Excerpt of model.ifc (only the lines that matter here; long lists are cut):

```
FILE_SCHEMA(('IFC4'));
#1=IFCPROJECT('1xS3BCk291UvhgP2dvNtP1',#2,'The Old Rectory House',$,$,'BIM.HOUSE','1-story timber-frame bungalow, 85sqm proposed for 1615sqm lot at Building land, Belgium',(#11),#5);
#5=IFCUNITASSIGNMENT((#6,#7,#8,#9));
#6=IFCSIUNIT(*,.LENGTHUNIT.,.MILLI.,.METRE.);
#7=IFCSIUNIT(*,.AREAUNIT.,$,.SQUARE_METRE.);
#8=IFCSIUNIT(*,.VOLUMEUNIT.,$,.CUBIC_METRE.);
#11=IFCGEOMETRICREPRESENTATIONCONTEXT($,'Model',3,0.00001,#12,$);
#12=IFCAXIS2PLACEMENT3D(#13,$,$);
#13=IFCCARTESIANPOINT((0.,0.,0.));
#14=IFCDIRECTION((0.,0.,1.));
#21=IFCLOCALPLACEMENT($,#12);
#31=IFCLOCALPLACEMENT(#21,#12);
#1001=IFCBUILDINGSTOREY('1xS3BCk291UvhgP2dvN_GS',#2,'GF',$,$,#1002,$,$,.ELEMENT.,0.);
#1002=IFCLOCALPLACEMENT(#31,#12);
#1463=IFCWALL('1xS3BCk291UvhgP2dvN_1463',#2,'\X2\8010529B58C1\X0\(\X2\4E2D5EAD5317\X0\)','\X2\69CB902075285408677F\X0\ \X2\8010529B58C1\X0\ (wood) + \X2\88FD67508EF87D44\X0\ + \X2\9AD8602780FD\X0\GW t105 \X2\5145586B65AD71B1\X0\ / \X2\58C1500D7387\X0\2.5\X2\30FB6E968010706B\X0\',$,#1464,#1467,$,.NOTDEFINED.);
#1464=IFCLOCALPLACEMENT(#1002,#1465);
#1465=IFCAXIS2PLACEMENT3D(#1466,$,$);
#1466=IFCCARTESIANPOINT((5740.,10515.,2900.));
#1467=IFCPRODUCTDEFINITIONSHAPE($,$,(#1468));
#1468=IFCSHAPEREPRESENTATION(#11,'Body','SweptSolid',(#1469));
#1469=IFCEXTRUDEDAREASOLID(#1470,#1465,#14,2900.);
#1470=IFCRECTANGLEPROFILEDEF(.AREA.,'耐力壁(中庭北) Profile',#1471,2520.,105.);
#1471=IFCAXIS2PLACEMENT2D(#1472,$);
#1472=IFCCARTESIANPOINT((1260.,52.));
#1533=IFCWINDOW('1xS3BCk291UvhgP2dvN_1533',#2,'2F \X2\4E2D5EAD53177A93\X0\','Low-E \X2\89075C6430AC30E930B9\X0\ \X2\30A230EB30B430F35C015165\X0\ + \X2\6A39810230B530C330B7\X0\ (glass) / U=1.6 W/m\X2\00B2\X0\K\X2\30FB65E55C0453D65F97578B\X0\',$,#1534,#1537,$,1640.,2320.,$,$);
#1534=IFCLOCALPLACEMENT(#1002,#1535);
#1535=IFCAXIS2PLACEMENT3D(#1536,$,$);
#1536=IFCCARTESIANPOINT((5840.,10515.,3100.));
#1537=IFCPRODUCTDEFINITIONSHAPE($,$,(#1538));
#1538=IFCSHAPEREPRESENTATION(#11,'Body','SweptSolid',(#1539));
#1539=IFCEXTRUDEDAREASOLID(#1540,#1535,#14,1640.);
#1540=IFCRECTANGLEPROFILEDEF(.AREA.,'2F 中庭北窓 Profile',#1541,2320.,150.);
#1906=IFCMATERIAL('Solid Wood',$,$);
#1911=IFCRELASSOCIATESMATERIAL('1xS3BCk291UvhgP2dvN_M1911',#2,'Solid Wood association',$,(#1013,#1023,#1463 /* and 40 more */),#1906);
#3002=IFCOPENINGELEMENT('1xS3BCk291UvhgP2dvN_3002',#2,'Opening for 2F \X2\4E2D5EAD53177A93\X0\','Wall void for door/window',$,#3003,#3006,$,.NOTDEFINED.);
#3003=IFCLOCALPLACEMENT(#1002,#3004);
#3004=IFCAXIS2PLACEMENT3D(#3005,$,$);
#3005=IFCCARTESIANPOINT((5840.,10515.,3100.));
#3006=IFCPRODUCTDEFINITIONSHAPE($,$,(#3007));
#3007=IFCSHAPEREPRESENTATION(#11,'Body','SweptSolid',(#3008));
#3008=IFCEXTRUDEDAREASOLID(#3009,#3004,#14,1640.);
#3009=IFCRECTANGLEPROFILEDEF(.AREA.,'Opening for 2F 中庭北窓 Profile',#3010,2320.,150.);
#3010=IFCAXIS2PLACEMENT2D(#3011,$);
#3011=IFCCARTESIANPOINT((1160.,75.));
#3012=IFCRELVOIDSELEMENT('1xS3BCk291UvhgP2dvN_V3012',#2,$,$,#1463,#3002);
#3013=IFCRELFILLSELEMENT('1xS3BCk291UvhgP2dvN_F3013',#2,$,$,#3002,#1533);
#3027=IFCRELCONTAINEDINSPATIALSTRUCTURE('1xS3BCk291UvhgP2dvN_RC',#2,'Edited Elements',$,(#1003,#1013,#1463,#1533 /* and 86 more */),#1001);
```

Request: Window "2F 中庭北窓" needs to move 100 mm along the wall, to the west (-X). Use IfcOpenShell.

```python
import ifcopenshell
import ifcopenshell.api.geometry
import ifcopenshell.util.placement
import ifcopenshell.util.unit

model = ifcopenshell.open("model.ifc")
unit_scale = ifcopenshell.util.unit.calculate_unit_scale(model)

window = model.by_guid("1xS3BCk291UvhgP2dvN_1533")
opening = window.FillsVoids[0].RelatingOpeningElement
wall = opening.VoidsElements[0].RelatingBuildingElement

wall_matrix = ifcopenshell.util.placement.get_local_placement(wall.ObjectPlacement)
shift = wall_matrix[:3, 0] * -0.1 / unit_scale
before = ifcopenshell.util.placement.get_local_placement(window.ObjectPlacement)[:3, 3].copy()

# The window is not placed relative to its opening, so move both.
for product in (opening, window):
    matrix = ifcopenshell.util.placement.get_local_placement(product.ObjectPlacement)
    matrix[:3, 3] += shift
    ifcopenshell.api.geometry.edit_object_placement(model, product=product, matrix=matrix, is_si=False)

after = ifcopenshell.util.placement.get_local_placement(window.ObjectPlacement)[:3, 3]
print("window moved by", (after - before).round(3) + 0.0)

model.write("model_v2.ifc")
```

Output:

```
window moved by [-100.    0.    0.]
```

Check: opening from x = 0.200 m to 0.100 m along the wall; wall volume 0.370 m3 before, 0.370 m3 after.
